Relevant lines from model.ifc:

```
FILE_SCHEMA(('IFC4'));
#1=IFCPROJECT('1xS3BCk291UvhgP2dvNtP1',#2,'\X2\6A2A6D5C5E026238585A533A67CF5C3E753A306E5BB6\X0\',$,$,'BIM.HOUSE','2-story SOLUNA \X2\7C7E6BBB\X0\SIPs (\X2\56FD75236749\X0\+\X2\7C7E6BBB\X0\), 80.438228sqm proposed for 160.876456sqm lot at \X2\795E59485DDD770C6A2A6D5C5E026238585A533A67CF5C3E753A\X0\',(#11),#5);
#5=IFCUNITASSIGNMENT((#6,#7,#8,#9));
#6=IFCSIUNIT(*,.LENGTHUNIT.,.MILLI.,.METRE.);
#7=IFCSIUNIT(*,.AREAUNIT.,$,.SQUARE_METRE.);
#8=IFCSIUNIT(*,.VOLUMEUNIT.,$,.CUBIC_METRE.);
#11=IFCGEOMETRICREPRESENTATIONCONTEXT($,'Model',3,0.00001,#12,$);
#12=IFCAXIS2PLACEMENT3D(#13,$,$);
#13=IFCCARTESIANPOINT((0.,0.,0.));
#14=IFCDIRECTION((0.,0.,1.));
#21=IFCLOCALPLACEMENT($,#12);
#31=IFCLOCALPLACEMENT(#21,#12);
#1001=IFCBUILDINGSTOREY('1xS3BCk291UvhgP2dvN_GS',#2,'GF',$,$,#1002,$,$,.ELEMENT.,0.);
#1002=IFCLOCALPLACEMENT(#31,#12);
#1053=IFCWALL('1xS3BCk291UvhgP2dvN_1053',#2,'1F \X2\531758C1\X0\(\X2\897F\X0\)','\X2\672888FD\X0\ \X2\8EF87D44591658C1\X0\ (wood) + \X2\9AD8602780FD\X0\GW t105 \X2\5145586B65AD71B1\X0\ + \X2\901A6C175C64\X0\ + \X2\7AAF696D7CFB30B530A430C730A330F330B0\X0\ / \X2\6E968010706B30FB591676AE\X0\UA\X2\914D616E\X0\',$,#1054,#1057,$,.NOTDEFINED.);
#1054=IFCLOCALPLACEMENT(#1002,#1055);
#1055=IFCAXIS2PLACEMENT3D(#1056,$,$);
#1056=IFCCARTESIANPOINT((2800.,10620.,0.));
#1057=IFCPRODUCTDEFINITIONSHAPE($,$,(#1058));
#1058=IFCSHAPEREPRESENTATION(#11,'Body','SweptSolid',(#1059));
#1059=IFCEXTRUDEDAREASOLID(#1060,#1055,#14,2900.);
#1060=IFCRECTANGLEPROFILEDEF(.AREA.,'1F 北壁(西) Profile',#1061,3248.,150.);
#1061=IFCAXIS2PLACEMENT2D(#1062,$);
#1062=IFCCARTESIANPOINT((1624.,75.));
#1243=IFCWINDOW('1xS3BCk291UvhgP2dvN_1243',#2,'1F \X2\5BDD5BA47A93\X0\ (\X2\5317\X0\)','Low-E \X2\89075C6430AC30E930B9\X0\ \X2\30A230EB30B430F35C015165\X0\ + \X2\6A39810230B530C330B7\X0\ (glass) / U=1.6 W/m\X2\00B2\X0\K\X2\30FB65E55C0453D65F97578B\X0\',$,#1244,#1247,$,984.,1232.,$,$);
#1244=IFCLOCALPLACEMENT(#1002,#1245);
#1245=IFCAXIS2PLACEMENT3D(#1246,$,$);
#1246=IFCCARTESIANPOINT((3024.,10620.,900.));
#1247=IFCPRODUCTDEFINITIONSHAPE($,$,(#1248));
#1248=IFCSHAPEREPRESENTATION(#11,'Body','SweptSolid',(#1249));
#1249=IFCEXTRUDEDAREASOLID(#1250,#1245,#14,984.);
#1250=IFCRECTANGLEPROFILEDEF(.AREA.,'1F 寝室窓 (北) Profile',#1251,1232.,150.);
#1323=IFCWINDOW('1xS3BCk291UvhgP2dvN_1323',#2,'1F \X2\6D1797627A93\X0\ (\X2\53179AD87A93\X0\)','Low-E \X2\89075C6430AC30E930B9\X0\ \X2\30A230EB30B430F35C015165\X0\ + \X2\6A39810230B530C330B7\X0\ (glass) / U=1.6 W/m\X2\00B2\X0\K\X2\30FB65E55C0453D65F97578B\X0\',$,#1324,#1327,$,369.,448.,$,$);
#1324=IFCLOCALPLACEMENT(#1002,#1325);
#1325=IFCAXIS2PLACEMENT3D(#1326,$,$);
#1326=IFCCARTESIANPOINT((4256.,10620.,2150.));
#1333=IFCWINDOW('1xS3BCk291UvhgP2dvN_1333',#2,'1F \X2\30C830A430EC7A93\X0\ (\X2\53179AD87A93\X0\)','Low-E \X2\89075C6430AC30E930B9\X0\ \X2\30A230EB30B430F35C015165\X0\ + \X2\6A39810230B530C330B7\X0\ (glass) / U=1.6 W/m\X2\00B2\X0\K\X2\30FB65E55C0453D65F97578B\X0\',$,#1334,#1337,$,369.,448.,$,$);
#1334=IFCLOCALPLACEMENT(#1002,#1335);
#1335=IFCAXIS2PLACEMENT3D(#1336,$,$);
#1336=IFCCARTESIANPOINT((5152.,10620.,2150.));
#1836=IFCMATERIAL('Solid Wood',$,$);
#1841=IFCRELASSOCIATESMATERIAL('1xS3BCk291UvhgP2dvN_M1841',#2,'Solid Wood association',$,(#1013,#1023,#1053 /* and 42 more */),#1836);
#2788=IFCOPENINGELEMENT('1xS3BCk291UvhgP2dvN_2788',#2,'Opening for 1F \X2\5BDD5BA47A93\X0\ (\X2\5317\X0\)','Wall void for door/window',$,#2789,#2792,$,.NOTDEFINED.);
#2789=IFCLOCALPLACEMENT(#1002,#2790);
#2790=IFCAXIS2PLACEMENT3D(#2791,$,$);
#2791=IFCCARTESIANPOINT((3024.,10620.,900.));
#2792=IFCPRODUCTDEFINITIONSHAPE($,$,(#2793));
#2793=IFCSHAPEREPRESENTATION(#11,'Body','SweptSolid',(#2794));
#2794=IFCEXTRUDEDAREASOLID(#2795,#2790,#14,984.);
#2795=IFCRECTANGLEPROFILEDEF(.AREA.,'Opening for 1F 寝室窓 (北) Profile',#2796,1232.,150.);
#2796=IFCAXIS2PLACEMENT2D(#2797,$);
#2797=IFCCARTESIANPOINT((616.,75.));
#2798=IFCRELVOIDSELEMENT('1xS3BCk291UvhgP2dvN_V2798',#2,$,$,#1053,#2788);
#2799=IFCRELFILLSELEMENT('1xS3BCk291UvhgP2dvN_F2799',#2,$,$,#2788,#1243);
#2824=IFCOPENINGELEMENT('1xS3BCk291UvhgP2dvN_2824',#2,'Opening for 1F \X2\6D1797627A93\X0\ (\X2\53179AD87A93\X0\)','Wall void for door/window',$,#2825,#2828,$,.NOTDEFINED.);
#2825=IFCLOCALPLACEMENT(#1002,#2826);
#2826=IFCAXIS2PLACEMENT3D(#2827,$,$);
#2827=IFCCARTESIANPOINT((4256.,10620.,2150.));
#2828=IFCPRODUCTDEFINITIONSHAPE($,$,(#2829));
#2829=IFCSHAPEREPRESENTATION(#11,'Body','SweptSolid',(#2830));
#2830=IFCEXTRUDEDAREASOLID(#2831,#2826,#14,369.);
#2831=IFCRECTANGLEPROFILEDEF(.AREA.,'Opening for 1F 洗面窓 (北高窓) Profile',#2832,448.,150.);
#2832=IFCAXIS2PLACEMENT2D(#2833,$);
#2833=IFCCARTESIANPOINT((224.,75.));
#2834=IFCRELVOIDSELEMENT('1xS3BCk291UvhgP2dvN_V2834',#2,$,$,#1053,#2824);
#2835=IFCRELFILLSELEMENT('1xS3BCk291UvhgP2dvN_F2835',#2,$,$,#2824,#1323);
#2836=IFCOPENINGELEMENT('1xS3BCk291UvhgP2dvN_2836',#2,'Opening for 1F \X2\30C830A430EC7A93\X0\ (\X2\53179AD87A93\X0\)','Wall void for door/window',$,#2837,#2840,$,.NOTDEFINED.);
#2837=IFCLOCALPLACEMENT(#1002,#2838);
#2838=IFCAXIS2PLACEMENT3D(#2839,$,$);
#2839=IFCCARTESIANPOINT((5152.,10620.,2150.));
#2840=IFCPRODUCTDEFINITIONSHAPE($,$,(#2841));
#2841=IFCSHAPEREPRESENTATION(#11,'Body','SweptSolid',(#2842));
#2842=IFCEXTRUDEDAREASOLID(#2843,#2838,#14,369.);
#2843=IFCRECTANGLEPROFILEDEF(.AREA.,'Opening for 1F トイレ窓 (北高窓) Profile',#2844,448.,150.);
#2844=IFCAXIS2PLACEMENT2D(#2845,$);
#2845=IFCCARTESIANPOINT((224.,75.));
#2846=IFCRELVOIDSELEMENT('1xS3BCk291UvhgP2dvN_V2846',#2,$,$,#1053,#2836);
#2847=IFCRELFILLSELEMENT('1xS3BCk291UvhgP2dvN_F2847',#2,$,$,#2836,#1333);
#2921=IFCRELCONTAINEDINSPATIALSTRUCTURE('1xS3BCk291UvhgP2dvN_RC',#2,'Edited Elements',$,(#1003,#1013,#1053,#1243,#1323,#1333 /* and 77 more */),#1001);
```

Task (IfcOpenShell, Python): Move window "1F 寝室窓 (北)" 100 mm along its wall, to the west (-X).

```python
import ifcopenshell
import ifcopenshell.api.geometry
import ifcopenshell.util.placement
import ifcopenshell.util.unit

model = ifcopenshell.open("model.ifc")
unit_scale = ifcopenshell.util.unit.calculate_unit_scale(model)

window = model.by_guid("1xS3BCk291UvhgP2dvN_1243")
opening = window.FillsVoids[0].RelatingOpeningElement
wall = opening.VoidsElements[0].RelatingBuildingElement

wall_matrix = ifcopenshell.util.placement.get_local_placement(wall.ObjectPlacement)
shift = wall_matrix[:3, 0] * -0.1 / unit_scale
before = ifcopenshell.util.placement.get_local_placement(window.ObjectPlacement)[:3, 3].copy()

# The window is not placed relative to its opening, so move both.
for product in (opening, window):
    matrix = ifcopenshell.util.placement.get_local_placement(product.ObjectPlacement)
    matrix[:3, 3] += shift
    ifcopenshell.api.geometry.edit_object_placement(model, product=product, matrix=matrix, is_si=False)

after = ifcopenshell.util.placement.get_local_placement(window.ObjectPlacement)[:3, 3]
print("window moved by", (after - before).round(3) + 0.0)

model.write("model_v2.ifc")
```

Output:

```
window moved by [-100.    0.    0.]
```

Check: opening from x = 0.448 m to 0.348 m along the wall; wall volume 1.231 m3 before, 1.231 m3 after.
